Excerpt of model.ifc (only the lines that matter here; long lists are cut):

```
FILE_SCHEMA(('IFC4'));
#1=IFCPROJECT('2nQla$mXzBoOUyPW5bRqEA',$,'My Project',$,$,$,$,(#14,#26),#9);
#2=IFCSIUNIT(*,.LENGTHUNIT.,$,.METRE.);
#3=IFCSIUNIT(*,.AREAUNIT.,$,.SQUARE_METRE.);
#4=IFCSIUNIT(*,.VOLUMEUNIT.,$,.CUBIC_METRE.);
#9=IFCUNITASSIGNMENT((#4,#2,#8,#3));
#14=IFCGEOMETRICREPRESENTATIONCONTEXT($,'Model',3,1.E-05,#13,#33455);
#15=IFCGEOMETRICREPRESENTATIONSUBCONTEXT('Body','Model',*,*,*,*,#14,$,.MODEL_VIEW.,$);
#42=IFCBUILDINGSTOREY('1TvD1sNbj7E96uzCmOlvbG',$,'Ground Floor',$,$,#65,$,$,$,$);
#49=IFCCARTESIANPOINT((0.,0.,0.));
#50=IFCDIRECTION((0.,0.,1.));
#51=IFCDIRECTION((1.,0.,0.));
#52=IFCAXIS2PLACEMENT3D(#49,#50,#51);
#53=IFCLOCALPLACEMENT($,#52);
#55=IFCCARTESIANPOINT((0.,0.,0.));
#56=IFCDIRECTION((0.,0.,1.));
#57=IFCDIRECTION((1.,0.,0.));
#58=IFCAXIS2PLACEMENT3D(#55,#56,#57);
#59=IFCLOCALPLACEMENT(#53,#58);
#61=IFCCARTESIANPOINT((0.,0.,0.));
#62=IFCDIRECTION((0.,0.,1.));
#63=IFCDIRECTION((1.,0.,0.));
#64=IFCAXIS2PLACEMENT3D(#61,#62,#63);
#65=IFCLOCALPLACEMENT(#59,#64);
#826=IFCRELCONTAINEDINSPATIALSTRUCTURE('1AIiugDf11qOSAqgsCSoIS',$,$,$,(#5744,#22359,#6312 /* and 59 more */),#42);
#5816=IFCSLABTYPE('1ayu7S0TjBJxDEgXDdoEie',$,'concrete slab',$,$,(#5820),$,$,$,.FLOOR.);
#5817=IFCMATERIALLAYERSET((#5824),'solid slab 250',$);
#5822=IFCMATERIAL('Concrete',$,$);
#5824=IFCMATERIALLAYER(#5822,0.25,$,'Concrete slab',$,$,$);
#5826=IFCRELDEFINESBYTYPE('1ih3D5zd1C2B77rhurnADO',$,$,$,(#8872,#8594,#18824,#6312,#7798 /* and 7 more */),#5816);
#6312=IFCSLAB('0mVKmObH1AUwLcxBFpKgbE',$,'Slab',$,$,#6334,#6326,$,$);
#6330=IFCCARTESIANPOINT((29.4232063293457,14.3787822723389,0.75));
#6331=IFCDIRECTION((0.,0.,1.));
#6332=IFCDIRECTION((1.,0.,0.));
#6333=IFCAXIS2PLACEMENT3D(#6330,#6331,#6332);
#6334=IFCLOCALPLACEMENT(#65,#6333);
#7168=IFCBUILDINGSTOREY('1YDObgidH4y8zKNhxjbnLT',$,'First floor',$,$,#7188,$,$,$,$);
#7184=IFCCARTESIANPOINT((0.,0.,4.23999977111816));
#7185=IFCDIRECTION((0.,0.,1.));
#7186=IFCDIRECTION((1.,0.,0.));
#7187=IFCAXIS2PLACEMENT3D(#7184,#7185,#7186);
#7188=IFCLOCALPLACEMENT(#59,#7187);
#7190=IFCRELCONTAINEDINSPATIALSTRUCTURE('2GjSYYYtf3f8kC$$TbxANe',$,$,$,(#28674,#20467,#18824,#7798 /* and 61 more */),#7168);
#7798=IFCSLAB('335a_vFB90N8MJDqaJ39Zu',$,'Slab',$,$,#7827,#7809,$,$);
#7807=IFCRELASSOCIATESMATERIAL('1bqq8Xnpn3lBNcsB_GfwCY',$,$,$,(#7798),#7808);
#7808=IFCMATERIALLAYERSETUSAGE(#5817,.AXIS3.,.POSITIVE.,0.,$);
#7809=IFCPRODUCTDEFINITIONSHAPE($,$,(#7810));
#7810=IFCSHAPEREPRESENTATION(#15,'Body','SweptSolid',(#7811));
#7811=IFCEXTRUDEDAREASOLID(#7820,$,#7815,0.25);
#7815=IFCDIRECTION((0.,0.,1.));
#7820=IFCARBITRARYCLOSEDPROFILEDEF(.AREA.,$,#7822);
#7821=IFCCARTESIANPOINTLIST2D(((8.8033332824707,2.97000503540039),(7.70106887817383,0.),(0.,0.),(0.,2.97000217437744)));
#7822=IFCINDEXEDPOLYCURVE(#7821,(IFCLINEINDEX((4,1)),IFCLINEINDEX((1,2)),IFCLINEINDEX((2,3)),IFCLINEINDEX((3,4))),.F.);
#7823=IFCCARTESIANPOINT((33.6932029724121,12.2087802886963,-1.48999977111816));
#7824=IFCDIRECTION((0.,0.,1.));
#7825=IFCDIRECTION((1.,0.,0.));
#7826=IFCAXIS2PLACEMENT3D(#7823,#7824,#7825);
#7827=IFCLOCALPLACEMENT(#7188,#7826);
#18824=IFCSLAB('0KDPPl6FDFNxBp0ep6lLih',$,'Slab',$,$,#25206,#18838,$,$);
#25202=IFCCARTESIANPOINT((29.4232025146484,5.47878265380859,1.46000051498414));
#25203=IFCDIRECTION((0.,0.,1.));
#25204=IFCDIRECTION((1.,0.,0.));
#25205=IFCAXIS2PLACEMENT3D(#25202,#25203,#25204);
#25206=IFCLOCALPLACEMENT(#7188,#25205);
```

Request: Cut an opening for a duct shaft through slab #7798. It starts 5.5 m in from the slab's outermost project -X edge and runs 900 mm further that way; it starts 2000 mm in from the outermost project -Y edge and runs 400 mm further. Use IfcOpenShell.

```python
import numpy as np
import ifcopenshell
import ifcopenshell.api.feature
import ifcopenshell.api.geometry
import ifcopenshell.api.root
import ifcopenshell.geom
import ifcopenshell.util.placement
import ifcopenshell.util.representation
import ifcopenshell.util.shape
import ifcopenshell.util.unit

model = ifcopenshell.open("model.ifc")
unit_scale = ifcopenshell.util.unit.calculate_unit_scale(model)
settings = ifcopenshell.geom.settings()


def volume(element):
    """Net volume in cubic metres, openings subtracted."""
    shape = ifcopenshell.geom.create_shape(settings, element)
    return ifcopenshell.util.shape.get_volume(shape.geometry)


slab = model.by_guid("335a_vFB90N8MJDqaJ39Zu")
before = volume(slab)

# Extent in the slab's own axes, in metres. The edges named are its -X and -Y sides.
slab_shape = ifcopenshell.geom.create_shape(settings, slab)
vertices = ifcopenshell.util.shape.get_vertices(slab_shape.geometry)
x_min, y_min, bottom = vertices.min(axis=0)
top = vertices[:, 2].max()

opening = ifcopenshell.api.root.create_entity(model, ifc_class="IfcOpeningElement", name="Duct shaft opening", predefined_type="OPENING")
context = ifcopenshell.util.representation.get_context(model, "Model", "Body", "MODEL_VIEW")
width, depth = 0.9, 0.4
outline = [(0.0, 0.0), (width, 0.0), (width, depth), (0.0, depth), (0.0, 0.0)]
# Overshoot both faces by 50 mm so the cut is clean.
shape = ifcopenshell.api.geometry.add_slab_representation(
    model, context=context, depth=top - bottom + 0.1, polyline=outline
)
ifcopenshell.api.geometry.assign_representation(model, product=opening, representation=shape)

matrix = ifcopenshell.util.placement.get_local_placement(slab.ObjectPlacement)
matrix[:, 3] = matrix @ np.append(np.array([x_min + 5.5, y_min + 2, bottom - 0.05]) / unit_scale, 1.0)
ifcopenshell.api.geometry.edit_object_placement(model, product=opening, matrix=matrix, is_si=False)
ifcopenshell.api.feature.add_feature(model, feature=opening, element=slab)

after = volume(slab)

print(f"slab volume {before:.3f} -> {after:.3f} m3")

model.write("model_rev.ifc")
```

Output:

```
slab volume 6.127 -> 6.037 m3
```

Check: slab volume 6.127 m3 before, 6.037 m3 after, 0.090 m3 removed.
